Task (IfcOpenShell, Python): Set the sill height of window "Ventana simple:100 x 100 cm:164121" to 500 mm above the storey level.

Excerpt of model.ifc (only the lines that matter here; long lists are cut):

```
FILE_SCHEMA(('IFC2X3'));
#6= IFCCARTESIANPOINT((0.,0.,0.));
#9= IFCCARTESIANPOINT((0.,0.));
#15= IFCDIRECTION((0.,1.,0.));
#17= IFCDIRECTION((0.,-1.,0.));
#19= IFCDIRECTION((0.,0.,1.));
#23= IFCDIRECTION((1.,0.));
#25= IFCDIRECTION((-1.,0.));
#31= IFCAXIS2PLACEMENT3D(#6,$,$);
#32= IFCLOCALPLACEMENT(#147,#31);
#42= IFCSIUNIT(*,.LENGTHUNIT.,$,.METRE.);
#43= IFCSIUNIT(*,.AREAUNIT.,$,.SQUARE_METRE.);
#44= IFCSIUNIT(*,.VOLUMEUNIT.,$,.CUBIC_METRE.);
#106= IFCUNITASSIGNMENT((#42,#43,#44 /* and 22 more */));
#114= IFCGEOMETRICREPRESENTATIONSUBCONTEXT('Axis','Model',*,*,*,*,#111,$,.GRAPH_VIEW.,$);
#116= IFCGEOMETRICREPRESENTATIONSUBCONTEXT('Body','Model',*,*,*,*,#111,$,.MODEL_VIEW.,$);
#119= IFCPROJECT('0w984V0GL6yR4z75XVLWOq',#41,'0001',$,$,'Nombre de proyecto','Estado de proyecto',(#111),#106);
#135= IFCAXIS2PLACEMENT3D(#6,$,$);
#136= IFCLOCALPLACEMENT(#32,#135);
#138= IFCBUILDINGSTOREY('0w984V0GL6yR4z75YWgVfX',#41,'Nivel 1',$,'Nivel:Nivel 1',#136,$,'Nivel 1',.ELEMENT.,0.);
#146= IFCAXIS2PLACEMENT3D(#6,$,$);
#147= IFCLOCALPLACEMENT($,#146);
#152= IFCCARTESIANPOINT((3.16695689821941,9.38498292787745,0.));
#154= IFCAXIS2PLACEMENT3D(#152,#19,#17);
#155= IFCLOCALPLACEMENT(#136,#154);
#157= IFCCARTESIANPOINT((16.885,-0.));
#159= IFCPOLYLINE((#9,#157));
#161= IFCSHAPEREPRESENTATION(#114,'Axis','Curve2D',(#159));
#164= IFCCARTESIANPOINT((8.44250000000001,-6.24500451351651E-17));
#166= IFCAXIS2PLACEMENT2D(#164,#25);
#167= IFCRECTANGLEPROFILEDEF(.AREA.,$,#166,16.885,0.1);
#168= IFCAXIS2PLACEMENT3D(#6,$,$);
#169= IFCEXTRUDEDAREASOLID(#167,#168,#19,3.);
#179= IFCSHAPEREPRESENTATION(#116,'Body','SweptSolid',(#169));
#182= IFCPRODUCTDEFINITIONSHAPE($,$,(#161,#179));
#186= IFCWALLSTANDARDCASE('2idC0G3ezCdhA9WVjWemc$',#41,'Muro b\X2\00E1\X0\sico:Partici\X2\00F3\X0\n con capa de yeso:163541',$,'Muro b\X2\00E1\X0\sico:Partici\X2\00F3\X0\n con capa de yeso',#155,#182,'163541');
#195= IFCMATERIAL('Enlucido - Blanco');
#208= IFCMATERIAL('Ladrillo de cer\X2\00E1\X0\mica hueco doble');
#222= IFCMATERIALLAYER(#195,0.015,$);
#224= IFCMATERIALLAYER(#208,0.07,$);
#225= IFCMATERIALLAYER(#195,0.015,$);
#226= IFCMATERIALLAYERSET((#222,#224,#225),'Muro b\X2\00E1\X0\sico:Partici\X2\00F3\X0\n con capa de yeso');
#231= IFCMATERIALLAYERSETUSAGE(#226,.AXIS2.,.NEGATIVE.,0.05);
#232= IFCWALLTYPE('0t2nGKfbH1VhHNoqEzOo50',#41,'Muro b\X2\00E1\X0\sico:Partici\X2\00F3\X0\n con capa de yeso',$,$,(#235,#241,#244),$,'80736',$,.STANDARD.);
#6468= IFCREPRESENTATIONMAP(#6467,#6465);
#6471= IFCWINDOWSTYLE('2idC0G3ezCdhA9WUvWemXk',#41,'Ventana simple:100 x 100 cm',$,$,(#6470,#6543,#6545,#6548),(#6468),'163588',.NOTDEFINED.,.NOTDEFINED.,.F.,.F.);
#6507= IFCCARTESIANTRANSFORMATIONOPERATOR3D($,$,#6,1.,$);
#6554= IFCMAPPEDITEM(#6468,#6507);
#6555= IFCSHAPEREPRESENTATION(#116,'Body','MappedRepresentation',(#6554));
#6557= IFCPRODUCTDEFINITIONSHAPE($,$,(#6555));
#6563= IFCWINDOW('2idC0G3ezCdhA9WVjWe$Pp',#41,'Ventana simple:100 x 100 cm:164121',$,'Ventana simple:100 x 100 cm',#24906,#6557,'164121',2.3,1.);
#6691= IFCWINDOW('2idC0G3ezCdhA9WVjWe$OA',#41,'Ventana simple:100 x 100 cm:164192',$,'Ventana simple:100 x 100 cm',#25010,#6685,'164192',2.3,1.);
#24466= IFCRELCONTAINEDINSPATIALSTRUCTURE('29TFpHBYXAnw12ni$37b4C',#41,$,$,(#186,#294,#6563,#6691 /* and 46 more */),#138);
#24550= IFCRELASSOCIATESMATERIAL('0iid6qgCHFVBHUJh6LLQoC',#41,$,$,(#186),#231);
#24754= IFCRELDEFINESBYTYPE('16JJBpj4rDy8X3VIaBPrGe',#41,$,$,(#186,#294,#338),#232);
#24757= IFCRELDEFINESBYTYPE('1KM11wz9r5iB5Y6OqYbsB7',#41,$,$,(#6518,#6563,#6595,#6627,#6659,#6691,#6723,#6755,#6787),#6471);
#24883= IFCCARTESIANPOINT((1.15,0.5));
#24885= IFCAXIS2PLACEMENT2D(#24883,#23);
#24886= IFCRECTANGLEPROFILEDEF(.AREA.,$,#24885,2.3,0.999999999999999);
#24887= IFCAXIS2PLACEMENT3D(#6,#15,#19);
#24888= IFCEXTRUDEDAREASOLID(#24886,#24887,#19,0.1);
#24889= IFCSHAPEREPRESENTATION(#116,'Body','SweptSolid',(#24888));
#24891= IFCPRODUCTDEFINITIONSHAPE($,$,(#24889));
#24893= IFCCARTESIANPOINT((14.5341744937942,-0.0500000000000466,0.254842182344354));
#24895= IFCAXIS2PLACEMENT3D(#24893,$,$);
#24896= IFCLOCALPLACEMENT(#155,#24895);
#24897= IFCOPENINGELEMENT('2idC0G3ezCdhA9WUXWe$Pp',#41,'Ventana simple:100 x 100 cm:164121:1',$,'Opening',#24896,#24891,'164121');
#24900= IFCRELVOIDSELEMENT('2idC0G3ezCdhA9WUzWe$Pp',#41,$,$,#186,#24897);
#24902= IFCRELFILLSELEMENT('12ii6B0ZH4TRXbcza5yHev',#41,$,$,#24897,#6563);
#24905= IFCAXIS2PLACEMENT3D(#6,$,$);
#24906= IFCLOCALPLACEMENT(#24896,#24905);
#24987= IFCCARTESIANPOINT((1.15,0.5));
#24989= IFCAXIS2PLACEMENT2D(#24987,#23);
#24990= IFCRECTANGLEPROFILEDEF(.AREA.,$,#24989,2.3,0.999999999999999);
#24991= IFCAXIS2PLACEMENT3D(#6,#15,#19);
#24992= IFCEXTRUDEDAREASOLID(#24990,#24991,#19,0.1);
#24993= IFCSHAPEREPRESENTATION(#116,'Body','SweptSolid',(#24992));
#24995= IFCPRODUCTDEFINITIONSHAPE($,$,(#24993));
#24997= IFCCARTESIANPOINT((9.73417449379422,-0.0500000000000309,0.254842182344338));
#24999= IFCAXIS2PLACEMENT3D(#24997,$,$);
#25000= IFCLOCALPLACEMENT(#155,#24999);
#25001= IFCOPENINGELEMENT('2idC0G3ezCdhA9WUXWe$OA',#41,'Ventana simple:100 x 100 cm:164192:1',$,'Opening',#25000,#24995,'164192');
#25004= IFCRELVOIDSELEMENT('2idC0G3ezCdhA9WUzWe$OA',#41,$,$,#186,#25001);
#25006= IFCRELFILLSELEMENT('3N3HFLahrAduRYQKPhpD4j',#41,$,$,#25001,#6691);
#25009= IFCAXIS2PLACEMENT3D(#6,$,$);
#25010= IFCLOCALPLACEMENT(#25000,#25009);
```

```python
import numpy as np
import ifcopenshell
import ifcopenshell.api.geometry
import ifcopenshell.geom
import ifcopenshell.util.element
import ifcopenshell.util.placement
import ifcopenshell.util.shape
import ifcopenshell.util.unit

model = ifcopenshell.open("model.ifc")
unit_scale = ifcopenshell.util.unit.calculate_unit_scale(model)

window = model.by_id(6563)
opening = window.FillsVoids[0].RelatingOpeningElement
storey = ifcopenshell.util.element.get_container(window, ifc_class="IfcBuildingStorey")
level = ifcopenshell.util.placement.get_local_placement(storey.ObjectPlacement)[2, 3]

# The opening's origin need not be at the sill, so measure its lowest point.
shape = ifcopenshell.geom.create_shape(ifcopenshell.geom.settings(), opening)
bottom = ifcopenshell.util.shape.get_shape_bottom_elevation(shape, shape.geometry) / unit_scale
dz = level + 0.5 / unit_scale - bottom

shift = np.array([0.0, 0.0, dz])
# The window is placed relative to its opening, so it follows when the opening moves.
matrix = ifcopenshell.util.placement.get_local_placement(opening.ObjectPlacement)
matrix[:3, 3] += shift
ifcopenshell.api.geometry.edit_object_placement(
    model, product=opening, matrix=matrix, is_si=False, should_transform_children=True
)

print(f"moved by {dz * unit_scale:+.3f} m")

model.write("model_v2.ifc")
```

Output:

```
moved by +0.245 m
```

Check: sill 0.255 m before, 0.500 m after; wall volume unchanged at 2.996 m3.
